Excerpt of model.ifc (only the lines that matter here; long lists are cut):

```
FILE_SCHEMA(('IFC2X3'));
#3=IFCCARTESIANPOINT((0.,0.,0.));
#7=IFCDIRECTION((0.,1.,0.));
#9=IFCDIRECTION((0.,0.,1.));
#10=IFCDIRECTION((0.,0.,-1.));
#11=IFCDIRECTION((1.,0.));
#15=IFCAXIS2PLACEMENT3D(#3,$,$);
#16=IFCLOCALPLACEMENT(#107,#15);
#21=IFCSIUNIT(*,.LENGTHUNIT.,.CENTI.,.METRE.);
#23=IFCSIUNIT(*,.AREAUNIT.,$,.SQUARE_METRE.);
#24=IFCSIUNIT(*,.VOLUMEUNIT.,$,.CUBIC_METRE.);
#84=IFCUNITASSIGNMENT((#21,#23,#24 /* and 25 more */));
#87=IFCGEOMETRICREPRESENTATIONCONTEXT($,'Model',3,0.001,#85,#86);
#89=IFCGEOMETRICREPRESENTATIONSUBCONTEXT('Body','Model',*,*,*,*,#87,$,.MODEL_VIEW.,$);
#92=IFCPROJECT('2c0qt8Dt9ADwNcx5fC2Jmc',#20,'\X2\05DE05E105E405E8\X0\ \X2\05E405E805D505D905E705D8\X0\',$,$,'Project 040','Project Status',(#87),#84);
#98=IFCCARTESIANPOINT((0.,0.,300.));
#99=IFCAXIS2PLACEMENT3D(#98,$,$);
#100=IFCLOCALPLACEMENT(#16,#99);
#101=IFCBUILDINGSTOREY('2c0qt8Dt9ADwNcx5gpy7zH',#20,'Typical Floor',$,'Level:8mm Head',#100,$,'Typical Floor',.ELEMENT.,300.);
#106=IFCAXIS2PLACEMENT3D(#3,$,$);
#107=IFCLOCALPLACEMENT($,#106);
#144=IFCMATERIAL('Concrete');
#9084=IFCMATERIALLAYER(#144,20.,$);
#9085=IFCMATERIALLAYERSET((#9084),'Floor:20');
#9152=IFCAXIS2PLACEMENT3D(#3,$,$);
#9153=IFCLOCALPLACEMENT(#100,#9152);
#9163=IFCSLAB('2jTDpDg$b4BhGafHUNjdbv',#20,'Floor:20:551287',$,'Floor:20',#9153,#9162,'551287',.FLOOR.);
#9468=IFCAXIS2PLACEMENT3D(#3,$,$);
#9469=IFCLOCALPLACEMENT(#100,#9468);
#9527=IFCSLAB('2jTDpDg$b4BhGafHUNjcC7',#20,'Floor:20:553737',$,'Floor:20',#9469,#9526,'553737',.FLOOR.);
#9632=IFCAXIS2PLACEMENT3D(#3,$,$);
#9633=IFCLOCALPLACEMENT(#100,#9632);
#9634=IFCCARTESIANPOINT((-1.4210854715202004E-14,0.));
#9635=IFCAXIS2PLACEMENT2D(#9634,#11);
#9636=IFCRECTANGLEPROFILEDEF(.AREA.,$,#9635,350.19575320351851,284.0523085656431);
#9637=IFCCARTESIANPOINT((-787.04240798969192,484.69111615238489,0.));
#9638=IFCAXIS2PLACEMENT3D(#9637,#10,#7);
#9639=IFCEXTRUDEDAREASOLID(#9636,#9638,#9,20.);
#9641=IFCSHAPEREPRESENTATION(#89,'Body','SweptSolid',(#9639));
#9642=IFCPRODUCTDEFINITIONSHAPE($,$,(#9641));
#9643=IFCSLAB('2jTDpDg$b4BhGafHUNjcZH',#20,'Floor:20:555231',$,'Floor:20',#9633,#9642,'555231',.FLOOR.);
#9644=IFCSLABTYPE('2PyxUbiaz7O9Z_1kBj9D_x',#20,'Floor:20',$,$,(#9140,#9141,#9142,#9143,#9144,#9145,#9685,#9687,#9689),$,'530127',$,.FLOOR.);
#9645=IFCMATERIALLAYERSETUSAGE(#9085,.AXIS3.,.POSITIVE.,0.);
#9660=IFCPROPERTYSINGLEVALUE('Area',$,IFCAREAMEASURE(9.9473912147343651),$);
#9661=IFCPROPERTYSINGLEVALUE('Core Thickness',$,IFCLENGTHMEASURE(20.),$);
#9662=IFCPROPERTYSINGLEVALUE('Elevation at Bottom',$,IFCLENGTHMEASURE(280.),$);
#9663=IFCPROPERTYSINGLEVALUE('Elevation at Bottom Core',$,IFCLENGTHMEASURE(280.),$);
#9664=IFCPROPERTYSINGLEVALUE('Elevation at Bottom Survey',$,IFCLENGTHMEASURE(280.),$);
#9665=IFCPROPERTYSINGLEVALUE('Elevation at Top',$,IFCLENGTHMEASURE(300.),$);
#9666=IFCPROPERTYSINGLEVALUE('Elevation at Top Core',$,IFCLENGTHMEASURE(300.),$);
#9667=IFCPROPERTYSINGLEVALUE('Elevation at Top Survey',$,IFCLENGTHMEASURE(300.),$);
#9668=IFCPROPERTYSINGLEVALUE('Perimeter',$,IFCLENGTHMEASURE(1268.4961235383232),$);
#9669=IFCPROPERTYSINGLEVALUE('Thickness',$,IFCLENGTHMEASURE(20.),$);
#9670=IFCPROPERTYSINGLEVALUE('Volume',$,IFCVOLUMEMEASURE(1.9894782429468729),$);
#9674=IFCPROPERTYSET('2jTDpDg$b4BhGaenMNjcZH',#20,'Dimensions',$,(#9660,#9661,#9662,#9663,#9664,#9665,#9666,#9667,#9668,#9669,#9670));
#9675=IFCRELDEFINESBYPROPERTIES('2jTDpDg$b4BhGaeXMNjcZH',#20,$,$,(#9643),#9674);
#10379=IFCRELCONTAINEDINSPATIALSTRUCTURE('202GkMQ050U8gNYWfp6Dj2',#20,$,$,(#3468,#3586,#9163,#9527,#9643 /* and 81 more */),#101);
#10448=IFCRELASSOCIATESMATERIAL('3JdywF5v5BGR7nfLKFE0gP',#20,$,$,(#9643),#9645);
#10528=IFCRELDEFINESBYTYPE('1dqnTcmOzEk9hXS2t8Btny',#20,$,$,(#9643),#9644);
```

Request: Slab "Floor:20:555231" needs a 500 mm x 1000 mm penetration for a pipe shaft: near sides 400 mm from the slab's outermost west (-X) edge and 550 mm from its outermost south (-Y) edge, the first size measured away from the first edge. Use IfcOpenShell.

```python
import numpy as np
import ifcopenshell
import ifcopenshell.api.feature
import ifcopenshell.api.geometry
import ifcopenshell.api.pset
import ifcopenshell.api.root
import ifcopenshell.geom
import ifcopenshell.util.element
import ifcopenshell.util.placement
import ifcopenshell.util.representation
import ifcopenshell.util.shape
import ifcopenshell.util.unit

model = ifcopenshell.open("model.ifc")
unit_scale = ifcopenshell.util.unit.calculate_unit_scale(model)
area_scale = ifcopenshell.util.unit.calculate_unit_scale(model, "AREAUNIT")
volume_scale = ifcopenshell.util.unit.calculate_unit_scale(model, "VOLUMEUNIT")
settings = ifcopenshell.geom.settings()


def volume(element):
    """Net volume in cubic metres, openings subtracted."""
    shape = ifcopenshell.geom.create_shape(settings, element)
    return ifcopenshell.util.shape.get_volume(shape.geometry)


slab = model.by_id(9643)
before = volume(slab)

# Extent in the slab's own axes, in metres. The edges named are its -X and -Y sides.
slab_shape = ifcopenshell.geom.create_shape(settings, slab)
vertices = ifcopenshell.util.shape.get_vertices(slab_shape.geometry)
x_min, y_min, bottom = vertices.min(axis=0)
top = vertices[:, 2].max()

opening = ifcopenshell.api.root.create_entity(model, ifc_class="IfcOpeningElement", name="Pipe shaft opening")
context = ifcopenshell.util.representation.get_context(model, "Model", "Body", "MODEL_VIEW")
width, depth = 0.5, 1
outline = [(0.0, 0.0), (width, 0.0), (width, depth), (0.0, depth), (0.0, 0.0)]
# Overshoot both faces by 50 mm so the cut is clean.
shape = ifcopenshell.api.geometry.add_slab_representation(
    model, context=context, depth=top - bottom + 0.1, polyline=outline
)
ifcopenshell.api.geometry.assign_representation(model, product=opening, representation=shape)

matrix = ifcopenshell.util.placement.get_local_placement(slab.ObjectPlacement)
matrix[:, 3] = matrix @ np.append(np.array([x_min + 0.4, y_min + 0.55, bottom - 0.05]) / unit_scale, 1.0)
ifcopenshell.api.geometry.edit_object_placement(model, product=opening, matrix=matrix, is_si=False)
ifcopenshell.api.feature.add_feature(model, feature=opening, element=slab)

after = volume(slab)

# Update the slab's stored quantities.
pset = model.by_id(ifcopenshell.util.element.get_pset(slab, "Dimensions", should_inherit=False)["id"])
ifcopenshell.api.pset.edit_pset(model, pset=pset, properties={
    "Area": model.create_entity("IfcAreaMeasure", after / (top - bottom) / area_scale),
    "Volume": model.create_entity("IfcVolumeMeasure", after / volume_scale),
})

print(f"slab volume {before:.3f} -> {after:.3f} m3")

model.write("model_edited.ifc")
```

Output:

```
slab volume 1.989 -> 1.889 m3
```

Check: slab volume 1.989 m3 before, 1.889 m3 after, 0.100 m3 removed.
